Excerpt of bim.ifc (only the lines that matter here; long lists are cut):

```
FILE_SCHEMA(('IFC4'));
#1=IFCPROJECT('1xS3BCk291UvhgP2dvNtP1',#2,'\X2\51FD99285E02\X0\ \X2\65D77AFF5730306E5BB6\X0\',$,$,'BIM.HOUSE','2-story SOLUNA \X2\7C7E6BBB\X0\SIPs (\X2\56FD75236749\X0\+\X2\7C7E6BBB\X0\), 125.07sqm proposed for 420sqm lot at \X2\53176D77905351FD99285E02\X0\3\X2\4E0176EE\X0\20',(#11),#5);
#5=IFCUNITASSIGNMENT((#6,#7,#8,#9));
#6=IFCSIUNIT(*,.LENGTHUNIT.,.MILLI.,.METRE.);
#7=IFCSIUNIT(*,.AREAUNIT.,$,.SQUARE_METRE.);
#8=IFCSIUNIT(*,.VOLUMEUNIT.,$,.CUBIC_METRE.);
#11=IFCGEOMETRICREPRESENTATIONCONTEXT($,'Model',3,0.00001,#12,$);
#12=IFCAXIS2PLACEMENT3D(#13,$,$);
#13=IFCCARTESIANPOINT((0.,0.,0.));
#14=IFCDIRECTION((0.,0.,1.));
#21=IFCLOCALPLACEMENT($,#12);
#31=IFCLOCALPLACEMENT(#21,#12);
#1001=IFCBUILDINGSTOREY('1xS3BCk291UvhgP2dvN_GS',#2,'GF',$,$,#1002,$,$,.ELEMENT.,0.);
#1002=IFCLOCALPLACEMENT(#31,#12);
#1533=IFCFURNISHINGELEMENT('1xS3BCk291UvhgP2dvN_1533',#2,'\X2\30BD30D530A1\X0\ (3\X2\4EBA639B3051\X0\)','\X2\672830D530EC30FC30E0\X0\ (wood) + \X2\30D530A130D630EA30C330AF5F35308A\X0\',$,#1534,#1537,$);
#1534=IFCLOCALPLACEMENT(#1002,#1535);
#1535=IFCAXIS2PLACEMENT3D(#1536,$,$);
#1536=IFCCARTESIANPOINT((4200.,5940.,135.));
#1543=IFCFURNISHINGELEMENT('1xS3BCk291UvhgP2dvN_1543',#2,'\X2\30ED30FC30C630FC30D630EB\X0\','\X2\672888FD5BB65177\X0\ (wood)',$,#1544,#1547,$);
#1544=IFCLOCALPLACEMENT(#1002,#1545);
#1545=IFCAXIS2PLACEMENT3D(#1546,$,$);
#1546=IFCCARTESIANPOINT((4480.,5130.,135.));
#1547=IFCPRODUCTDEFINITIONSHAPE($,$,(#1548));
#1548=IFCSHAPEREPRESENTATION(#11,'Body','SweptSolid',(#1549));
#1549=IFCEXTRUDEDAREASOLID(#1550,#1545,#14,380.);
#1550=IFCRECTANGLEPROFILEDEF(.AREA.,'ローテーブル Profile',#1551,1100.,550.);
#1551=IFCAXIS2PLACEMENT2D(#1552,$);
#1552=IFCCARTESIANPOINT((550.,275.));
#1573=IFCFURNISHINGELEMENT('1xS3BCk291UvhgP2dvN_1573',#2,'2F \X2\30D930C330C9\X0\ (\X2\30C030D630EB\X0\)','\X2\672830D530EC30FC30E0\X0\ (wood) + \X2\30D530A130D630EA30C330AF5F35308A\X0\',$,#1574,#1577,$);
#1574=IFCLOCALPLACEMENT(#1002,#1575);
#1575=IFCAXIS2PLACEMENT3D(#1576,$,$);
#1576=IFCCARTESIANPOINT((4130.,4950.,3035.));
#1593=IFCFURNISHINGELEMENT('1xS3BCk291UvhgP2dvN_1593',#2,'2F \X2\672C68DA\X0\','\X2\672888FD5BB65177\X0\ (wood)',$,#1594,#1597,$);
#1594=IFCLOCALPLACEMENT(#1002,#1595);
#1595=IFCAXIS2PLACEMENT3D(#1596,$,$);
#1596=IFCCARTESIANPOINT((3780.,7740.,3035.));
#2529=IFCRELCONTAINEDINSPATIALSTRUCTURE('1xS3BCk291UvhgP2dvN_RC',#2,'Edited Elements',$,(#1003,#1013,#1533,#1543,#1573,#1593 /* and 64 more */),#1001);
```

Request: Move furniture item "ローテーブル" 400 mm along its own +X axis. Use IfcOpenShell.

```python
import ifcopenshell
import ifcopenshell.api.geometry
import ifcopenshell.util.placement
import ifcopenshell.util.unit

model = ifcopenshell.open("bim.ifc")
unit_scale = ifcopenshell.util.unit.calculate_unit_scale(model)

item = model.by_id(1543)
matrix = ifcopenshell.util.placement.get_local_placement(item.ObjectPlacement)
matrix[:3, 3] += matrix[:3, 0] * 0.4 / unit_scale
ifcopenshell.api.geometry.edit_object_placement(model, product=item, matrix=matrix, is_si=False)

print(ifcopenshell.util.placement.get_local_placement(item.ObjectPlacement).round(3) + 0.0)

model.write("bim-out.ifc")
```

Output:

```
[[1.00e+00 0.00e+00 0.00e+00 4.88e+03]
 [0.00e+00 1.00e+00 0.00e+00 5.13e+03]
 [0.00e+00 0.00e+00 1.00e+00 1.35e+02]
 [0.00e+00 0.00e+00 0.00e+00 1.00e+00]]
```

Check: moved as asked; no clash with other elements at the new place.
